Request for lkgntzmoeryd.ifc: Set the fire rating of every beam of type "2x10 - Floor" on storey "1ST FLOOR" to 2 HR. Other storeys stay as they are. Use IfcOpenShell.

First a look at what the model holds.

```python
import ifcopenshell
import ifcopenshell.util.element

model = ifcopenshell.open("lkgntzmoeryd.ifc")
print(model.schema)
storey = next(s for s in model.by_type("IfcBuildingStorey") if s.Name == "1ST FLOOR")
beams = [e for e in ifcopenshell.util.element.get_decomposition(storey) if e.is_a("IfcBeam")]
seen = {}
for e in beams:
    element_type = ifcopenshell.util.element.get_type(e)
    key = (element_type.Name if element_type != e and element_type else None, ifcopenshell.util.element.get_pset(e, "Pset_BeamCommon", "FireRating"))
    seen[key] = seen.get(key, 0) + 1
for (name, value), count in sorted(seen.items(), key=str):
    print(count, "x", name, "|", value)
```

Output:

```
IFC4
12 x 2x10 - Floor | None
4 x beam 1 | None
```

```python
import ifcopenshell
import ifcopenshell.api.pset
import ifcopenshell.util.element

model = ifcopenshell.open("lkgntzmoeryd.ifc")

storey = next(s for s in model.by_type("IfcBuildingStorey") if s.Name == "1ST FLOOR")
beams = [e for e in ifcopenshell.util.element.get_decomposition(storey) if e.is_a("IfcBeam")]

count = 0
for e in beams:
    element_type = ifcopenshell.util.element.get_type(e)
    if element_type in (None, e) or element_type.Name != "2x10 - Floor":
        continue
    # add_pset returns the element's existing set when there is one.
    pset = ifcopenshell.api.pset.add_pset(model, product=e, name="Pset_BeamCommon")
    ifcopenshell.api.pset.edit_pset(model, pset=pset, properties={"FireRating": "2 HR"})
    count += 1

print(count, "beams updated")

model.write("lkgntzmoeryd_v2.ifc")
```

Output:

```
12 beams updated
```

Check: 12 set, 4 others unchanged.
